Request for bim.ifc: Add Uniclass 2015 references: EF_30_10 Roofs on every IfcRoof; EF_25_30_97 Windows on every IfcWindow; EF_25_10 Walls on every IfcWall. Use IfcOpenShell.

First a look at what the model holds.

```python
import ifcopenshell

model = ifcopenshell.open("bim.ifc")
print(model.schema)
print("classifications:", [c.Name for c in model.by_type("IfcClassification")])
for ifc_class in ("IfcDoor", "IfcRoof", "IfcStair", "IfcWall", "IfcWindow"):
    print(ifc_class, len(model.by_type(ifc_class)))
```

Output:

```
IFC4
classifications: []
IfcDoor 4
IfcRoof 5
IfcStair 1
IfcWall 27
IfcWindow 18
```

```python
import ifcopenshell
import ifcopenshell.api.classification

model = ifcopenshell.open("bim.ifc")

system = ifcopenshell.api.classification.add_classification(model, classification="Uniclass 2015")

codes = {
    "IfcRoof": ("EF_30_10", "Roofs"),
    "IfcWindow": ("EF_25_30_97", "Windows"),
    "IfcWall": ("EF_25_10", "Walls"),
}
for ifc_class, (code, name) in codes.items():
    products = model.by_type(ifc_class)
    ifcopenshell.api.classification.add_reference(
        model, products=products, classification=system, identification=code, name=name
    )
    print(code, len(products))

model.write("bim-out.ifc")
```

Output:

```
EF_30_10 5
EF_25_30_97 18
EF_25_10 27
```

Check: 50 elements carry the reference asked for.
